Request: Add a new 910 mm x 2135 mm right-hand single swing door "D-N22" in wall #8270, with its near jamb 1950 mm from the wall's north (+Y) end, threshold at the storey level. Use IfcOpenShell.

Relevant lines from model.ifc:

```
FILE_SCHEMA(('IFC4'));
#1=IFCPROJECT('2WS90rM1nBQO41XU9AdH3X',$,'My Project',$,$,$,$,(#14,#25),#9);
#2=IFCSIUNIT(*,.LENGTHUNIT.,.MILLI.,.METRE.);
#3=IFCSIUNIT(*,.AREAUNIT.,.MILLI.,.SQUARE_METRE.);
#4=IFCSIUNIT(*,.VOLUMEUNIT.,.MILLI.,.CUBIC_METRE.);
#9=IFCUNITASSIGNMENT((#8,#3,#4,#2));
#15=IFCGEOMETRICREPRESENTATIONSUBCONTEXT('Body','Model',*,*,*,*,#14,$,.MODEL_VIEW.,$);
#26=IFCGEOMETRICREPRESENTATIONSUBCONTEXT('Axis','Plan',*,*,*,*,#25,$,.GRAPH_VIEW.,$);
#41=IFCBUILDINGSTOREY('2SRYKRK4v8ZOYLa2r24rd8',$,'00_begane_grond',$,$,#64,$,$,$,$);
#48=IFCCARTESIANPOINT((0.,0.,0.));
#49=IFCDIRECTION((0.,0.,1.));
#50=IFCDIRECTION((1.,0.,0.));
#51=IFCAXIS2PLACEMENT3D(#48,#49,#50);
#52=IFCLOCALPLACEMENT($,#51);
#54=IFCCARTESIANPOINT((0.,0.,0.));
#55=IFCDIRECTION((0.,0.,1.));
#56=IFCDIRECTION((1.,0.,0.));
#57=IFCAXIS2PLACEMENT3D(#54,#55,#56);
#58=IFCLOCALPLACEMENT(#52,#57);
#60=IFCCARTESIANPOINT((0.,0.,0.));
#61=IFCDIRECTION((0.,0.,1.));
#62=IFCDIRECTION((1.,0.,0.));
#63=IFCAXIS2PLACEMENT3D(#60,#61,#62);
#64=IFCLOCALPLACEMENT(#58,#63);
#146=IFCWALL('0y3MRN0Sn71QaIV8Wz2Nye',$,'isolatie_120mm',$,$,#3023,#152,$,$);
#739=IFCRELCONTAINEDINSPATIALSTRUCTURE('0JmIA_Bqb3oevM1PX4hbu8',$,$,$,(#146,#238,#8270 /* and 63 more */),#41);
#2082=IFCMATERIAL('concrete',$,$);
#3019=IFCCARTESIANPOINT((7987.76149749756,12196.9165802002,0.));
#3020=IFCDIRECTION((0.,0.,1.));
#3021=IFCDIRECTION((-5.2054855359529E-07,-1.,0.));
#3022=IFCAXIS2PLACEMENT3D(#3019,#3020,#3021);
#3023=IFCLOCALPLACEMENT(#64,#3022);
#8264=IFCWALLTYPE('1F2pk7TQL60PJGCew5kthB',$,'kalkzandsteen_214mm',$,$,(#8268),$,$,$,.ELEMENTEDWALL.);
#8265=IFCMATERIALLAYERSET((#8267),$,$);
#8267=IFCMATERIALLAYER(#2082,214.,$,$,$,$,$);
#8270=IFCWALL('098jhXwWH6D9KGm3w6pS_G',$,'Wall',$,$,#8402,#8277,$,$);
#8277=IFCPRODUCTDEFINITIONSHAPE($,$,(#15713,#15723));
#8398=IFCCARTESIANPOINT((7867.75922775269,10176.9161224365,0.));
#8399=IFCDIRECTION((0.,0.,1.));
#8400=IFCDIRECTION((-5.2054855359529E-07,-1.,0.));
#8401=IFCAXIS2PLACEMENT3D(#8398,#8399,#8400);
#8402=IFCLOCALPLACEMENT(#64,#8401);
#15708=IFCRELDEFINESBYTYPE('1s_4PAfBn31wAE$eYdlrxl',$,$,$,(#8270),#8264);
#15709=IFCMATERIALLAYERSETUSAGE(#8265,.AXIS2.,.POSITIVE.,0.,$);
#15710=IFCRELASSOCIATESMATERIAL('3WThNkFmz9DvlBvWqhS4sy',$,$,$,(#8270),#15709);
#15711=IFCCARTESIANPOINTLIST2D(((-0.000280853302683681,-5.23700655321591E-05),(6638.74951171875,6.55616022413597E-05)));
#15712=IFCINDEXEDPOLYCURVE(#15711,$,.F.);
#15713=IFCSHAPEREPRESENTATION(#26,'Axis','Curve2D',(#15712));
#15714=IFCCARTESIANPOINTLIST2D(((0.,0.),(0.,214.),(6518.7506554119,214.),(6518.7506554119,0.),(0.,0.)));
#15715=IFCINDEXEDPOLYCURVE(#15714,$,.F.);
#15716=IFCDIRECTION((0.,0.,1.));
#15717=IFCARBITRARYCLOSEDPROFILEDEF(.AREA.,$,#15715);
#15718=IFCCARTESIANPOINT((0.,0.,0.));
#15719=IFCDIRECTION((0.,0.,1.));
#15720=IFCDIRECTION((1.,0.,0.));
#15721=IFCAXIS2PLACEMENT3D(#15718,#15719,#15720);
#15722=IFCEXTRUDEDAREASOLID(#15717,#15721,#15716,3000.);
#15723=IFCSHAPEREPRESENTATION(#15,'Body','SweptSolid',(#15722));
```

```python
import numpy as np
import ifcopenshell
import ifcopenshell.api.feature
import ifcopenshell.api.geometry
import ifcopenshell.api.root
import ifcopenshell.api.spatial
import ifcopenshell.geom
import ifcopenshell.util.element
import ifcopenshell.util.placement
import ifcopenshell.util.representation
import ifcopenshell.util.shape
import ifcopenshell.util.unit

model = ifcopenshell.open("model.ifc")
unit_scale = ifcopenshell.util.unit.calculate_unit_scale(model)
settings = ifcopenshell.geom.settings()


def volume(element):
    """Net volume in cubic metres, openings subtracted."""
    shape = ifcopenshell.geom.create_shape(settings, element)
    return ifcopenshell.util.shape.get_volume(shape.geometry)


wall = model.by_guid("098jhXwWH6D9KGm3w6pS_G")
storey = ifcopenshell.util.element.get_container(wall, ifc_class="IfcBuildingStorey")
context = ifcopenshell.util.representation.get_context(model, "Model", "Body", "MODEL_VIEW")
before = volume(wall)

width, height, from_end, sill = 0.91, 2.135, 1.95, 0.0  # metres

# The wall runs along its own X axis, and the end named is its -X end.
wall_shape = ifcopenshell.geom.create_shape(settings, wall)
x, y, z = ifcopenshell.util.shape.get_vertices(wall_shape.geometry).T
start = x.min() + from_end
face, thickness = float(y.min()), float(y.max() - y.min())
wall_matrix = ifcopenshell.util.placement.get_local_placement(wall.ObjectPlacement)
level = ifcopenshell.util.placement.get_local_placement(storey.ObjectPlacement)[2, 3]


def in_wall(x, y):
    """Placement at x, y metres in the wall's axes, at sill height."""
    matrix = wall_matrix.copy()
    matrix[:, 3] = wall_matrix @ np.array([x / unit_scale, y / unit_scale, 0.0, 1.0])
    matrix[2, 3] = level + sill / unit_scale
    return matrix


# Opening: a box that overshoots both wall faces by 50 mm.
opening = ifcopenshell.api.root.create_entity(model, ifc_class="IfcOpeningElement", predefined_type="OPENING")
box = ifcopenshell.api.geometry.add_wall_representation(
    model, context=context, length=width, height=height, thickness=thickness + 0.1
)
ifcopenshell.api.geometry.assign_representation(model, product=opening, representation=box)
ifcopenshell.api.geometry.edit_object_placement(model, product=opening, matrix=in_wall(start, face - 0.05), is_si=False)
ifcopenshell.api.feature.add_feature(model, feature=opening, element=wall)

door = ifcopenshell.api.root.create_entity(model, ifc_class="IfcDoor", name="D-N22", predefined_type="DOOR")
door.OverallWidth, door.OverallHeight = width / unit_scale, height / unit_scale
door.OperationType = "SINGLE_SWING_RIGHT"
body = ifcopenshell.api.geometry.add_door_representation(
    model,
    context=context,
    overall_width=door.OverallWidth,
    overall_height=door.OverallHeight,
    operation_type="SINGLE_SWING_RIGHT",
    lining_properties={"LiningDepth": thickness / unit_scale, "ThresholdDepth": thickness / unit_scale},
)
ifcopenshell.api.geometry.assign_representation(model, product=door, representation=body)
ifcopenshell.api.spatial.assign_container(model, products=[door], relating_structure=storey)
ifcopenshell.api.feature.add_filling(model, opening=opening, element=door)

# The lining spans the wall, so the door starts at the wall face.
ifcopenshell.api.geometry.edit_object_placement(model, product=door, matrix=in_wall(start, face), is_si=False)

after = volume(wall)

print(f"wall volume {before:.3f} -> {after:.3f} m3")

model.write("model_v2.ifc")
```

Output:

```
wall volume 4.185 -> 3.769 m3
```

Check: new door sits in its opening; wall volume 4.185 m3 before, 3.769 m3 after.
